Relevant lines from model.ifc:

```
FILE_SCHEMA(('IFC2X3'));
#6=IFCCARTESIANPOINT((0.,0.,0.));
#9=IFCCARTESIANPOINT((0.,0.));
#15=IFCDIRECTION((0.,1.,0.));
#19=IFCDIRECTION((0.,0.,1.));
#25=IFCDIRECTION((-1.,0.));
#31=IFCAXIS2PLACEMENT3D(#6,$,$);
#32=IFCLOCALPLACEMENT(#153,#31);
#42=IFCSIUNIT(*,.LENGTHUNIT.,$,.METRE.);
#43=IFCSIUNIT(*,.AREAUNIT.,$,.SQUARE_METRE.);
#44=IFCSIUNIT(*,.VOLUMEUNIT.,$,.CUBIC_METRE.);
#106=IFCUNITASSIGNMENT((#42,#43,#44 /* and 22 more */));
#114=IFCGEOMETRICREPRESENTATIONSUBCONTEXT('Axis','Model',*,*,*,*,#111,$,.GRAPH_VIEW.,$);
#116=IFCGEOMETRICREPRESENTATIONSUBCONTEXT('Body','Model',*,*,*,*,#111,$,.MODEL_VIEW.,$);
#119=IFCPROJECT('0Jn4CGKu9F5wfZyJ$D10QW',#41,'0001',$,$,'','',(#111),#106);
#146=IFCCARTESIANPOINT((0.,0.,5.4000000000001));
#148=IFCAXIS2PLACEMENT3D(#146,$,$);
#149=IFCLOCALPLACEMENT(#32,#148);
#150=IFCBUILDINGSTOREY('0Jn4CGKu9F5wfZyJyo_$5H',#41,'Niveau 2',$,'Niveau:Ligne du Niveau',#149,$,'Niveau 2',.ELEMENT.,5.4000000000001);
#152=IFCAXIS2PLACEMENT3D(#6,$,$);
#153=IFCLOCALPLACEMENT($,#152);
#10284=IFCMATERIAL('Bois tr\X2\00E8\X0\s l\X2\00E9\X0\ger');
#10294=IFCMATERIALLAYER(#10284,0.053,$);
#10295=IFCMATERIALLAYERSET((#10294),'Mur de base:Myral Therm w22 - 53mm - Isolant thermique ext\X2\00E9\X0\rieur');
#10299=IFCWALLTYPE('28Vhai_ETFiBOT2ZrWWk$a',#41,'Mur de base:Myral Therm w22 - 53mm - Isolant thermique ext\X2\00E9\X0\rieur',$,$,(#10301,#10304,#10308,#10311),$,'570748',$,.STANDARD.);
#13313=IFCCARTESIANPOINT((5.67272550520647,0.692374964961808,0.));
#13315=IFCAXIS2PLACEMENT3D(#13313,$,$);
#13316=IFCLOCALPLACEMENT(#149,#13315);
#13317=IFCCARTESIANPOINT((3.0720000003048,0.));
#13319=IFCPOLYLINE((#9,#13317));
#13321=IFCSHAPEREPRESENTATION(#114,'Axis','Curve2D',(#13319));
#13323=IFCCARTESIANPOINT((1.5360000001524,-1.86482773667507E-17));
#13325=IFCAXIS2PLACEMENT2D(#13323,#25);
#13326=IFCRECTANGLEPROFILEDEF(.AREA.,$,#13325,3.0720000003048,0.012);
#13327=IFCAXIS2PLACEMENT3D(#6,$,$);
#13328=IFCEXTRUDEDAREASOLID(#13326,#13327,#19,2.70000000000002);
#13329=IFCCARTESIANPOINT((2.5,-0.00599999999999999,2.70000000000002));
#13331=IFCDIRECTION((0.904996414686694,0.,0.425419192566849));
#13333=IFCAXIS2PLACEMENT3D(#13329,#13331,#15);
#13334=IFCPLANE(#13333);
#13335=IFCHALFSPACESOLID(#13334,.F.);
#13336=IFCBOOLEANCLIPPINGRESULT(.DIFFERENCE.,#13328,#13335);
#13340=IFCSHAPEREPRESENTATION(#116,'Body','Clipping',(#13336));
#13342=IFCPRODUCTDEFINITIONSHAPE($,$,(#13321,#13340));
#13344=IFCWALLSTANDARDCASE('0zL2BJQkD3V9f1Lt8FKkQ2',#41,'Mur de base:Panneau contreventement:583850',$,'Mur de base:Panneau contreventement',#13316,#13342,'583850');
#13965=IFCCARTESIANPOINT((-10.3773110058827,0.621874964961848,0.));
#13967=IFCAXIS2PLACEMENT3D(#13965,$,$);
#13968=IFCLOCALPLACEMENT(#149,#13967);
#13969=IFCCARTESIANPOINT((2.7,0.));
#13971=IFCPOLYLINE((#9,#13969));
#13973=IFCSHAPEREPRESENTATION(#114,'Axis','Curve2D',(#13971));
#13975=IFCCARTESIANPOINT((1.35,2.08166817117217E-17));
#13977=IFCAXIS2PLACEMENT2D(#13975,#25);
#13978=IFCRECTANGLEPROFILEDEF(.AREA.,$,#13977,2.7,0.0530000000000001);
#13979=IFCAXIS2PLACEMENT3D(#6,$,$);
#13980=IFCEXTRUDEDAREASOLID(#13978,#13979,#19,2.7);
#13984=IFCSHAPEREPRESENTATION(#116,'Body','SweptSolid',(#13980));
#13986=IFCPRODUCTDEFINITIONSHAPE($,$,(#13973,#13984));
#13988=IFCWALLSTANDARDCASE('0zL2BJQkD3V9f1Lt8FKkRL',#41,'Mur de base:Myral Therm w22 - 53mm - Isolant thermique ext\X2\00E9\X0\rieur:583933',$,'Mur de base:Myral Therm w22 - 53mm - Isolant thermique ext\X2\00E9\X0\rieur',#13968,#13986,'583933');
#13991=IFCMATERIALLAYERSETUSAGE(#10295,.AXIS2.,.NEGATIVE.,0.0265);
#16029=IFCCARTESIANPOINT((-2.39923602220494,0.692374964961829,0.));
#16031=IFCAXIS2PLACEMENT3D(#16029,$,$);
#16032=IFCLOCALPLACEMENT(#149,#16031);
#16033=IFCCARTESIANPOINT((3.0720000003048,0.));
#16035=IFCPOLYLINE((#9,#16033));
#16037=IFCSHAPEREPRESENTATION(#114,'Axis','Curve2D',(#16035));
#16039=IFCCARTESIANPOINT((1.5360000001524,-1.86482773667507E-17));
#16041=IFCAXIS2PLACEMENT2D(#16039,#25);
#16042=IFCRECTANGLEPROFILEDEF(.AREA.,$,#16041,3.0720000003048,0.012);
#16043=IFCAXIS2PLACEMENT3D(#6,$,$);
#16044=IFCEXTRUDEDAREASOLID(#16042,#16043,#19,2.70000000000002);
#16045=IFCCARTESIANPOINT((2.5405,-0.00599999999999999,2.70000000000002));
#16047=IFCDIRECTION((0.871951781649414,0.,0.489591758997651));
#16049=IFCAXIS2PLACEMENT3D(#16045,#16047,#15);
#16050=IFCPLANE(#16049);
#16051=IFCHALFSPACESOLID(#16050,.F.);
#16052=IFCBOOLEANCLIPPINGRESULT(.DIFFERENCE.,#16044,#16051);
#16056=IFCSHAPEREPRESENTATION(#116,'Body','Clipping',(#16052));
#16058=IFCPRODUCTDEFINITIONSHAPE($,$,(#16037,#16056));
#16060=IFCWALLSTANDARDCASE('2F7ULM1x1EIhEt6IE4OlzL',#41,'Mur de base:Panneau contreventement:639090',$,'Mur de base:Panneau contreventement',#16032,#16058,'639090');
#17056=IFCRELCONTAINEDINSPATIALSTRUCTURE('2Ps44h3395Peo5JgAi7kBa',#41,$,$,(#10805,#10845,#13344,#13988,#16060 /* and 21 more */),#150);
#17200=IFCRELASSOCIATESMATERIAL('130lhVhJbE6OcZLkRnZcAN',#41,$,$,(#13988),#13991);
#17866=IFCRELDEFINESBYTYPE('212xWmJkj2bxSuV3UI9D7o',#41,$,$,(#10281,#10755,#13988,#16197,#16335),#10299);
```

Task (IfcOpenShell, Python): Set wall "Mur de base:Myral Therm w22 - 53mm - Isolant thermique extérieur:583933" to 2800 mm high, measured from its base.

```python
import ifcopenshell
import ifcopenshell.geom
import ifcopenshell.util.representation
import ifcopenshell.util.shape
import ifcopenshell.util.unit

model = ifcopenshell.open("model.ifc")
unit_scale = ifcopenshell.util.unit.calculate_unit_scale(model)
settings = ifcopenshell.geom.settings()


def volume(element):
    """Net volume in cubic metres, openings subtracted."""
    shape = ifcopenshell.geom.create_shape(settings, element)
    return ifcopenshell.util.shape.get_volume(shape.geometry)


wall = model.by_id(13988)
before = volume(wall)

body = ifcopenshell.util.representation.get_representation(wall, "Model", "Body")
solid = body.Items[0]
old_height = solid.Depth
solid.Depth = 2.8 / unit_scale
after = volume(wall)

print(f"height {old_height:g} -> {solid.Depth:g}, volume {before:.3f} -> {after:.3f} m3")

model.write("model_edited.ifc")
```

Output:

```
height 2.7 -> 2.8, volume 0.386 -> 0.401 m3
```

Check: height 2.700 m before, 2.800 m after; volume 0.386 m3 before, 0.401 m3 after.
